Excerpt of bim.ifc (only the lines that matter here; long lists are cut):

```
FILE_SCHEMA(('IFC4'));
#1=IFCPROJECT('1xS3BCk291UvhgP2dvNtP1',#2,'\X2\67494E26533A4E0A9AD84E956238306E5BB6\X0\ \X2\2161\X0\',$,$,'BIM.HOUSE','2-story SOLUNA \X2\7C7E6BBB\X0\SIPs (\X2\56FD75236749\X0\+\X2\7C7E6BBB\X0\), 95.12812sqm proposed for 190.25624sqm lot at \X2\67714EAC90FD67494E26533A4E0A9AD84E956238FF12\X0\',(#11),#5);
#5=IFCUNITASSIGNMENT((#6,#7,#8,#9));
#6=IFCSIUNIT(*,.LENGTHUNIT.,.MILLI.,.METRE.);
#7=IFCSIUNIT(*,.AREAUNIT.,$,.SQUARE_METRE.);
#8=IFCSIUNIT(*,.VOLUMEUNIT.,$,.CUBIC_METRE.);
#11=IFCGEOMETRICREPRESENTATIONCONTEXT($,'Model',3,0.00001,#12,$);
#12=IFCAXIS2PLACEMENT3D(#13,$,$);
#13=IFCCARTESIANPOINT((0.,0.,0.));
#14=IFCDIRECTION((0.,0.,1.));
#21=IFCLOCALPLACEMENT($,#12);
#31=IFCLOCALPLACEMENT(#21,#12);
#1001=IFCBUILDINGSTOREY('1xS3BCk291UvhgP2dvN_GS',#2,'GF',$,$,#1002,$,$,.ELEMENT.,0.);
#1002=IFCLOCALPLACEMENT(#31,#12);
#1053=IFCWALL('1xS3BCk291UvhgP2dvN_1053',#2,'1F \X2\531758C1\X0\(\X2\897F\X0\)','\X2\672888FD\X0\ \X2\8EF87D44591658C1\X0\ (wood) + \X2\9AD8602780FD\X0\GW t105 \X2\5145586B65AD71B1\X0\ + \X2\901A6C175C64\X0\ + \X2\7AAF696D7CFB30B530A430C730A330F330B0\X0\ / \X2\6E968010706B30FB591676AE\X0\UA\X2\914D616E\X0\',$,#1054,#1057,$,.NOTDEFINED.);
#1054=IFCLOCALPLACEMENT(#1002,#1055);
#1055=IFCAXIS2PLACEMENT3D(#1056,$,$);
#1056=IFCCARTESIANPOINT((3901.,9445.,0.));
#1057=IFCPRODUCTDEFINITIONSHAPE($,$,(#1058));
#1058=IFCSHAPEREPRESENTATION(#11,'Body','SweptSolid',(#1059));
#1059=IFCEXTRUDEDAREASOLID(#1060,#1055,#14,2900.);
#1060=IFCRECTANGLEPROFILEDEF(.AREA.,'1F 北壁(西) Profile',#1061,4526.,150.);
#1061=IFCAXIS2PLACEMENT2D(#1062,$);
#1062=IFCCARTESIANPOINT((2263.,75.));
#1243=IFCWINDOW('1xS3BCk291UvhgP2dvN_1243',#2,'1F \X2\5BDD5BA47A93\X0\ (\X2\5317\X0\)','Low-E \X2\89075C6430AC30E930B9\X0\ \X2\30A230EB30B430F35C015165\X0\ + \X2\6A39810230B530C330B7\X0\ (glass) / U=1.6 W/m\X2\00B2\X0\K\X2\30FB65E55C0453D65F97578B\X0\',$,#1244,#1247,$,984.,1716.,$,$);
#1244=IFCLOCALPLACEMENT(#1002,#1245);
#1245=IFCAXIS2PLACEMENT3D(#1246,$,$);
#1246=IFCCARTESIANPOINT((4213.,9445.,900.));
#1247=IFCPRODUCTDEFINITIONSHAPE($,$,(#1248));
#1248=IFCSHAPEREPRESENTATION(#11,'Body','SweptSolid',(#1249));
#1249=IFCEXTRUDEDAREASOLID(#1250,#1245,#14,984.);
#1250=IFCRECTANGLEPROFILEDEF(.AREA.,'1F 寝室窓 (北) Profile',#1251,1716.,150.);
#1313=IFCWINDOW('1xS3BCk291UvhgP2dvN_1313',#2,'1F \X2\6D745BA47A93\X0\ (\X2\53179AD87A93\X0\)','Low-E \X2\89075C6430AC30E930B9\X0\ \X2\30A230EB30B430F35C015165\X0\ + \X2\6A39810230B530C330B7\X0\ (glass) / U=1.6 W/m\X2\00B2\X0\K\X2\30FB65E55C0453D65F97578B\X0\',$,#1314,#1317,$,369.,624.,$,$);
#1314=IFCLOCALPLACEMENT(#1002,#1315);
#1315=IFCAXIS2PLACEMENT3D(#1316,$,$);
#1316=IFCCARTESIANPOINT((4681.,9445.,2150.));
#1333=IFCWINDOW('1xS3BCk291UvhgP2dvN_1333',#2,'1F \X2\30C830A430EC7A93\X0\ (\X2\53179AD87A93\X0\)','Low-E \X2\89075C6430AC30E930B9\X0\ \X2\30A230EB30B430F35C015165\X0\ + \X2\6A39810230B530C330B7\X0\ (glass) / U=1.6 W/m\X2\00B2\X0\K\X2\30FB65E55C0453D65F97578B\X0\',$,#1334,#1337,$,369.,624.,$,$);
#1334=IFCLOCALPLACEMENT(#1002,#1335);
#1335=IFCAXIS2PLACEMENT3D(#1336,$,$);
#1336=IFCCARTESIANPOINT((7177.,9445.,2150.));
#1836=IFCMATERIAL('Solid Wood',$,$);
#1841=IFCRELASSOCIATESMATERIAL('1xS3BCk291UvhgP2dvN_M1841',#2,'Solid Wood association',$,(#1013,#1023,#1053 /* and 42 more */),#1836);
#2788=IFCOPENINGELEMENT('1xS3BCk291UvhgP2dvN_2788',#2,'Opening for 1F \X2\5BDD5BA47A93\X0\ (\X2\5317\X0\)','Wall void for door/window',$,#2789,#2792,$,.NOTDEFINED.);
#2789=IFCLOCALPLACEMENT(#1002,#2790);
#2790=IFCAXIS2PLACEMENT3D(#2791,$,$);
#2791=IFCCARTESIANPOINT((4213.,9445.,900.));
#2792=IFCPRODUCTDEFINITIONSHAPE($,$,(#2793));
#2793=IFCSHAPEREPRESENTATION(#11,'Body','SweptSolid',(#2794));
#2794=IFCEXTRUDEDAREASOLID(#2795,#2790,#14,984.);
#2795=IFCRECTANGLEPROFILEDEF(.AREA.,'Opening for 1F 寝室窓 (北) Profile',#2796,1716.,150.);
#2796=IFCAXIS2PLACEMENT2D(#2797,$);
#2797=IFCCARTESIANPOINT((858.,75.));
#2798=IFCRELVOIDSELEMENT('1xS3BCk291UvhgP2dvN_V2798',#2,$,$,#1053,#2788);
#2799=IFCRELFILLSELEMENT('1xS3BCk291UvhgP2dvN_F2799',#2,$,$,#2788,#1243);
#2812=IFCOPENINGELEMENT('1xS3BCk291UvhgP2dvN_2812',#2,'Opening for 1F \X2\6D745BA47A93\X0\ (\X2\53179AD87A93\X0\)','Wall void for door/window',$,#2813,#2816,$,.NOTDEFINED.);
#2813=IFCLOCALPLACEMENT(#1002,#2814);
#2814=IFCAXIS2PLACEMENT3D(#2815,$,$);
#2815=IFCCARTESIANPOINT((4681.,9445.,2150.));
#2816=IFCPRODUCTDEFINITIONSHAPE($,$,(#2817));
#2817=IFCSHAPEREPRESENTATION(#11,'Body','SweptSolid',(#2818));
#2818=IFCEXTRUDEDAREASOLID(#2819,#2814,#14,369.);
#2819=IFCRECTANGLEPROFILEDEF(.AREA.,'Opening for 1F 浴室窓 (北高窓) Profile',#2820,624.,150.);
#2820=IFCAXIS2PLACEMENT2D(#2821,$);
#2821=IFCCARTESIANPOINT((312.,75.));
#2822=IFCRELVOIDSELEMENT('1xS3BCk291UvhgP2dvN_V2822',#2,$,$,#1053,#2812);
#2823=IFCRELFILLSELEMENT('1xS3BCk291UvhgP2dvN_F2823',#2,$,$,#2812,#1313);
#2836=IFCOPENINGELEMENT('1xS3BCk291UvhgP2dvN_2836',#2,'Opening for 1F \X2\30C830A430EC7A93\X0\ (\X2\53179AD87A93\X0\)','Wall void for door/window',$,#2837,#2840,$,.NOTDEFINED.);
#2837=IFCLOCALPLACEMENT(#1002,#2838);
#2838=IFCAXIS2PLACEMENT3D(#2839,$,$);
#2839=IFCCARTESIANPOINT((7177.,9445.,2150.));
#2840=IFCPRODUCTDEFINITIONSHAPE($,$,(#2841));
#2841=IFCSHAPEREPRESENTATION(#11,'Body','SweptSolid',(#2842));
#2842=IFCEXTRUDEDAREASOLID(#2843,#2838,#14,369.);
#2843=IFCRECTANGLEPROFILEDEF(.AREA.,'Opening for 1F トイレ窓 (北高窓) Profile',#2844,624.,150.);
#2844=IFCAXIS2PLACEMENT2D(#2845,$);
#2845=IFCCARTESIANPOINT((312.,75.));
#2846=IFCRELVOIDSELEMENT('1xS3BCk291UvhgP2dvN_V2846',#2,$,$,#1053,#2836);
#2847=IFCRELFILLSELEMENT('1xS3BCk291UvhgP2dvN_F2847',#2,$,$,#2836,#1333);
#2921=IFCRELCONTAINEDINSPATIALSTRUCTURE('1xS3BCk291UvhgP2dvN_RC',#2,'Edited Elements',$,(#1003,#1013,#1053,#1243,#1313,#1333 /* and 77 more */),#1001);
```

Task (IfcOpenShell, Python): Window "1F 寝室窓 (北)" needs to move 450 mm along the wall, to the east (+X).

```python
import ifcopenshell
import ifcopenshell.api.geometry
import ifcopenshell.util.placement

model = ifcopenshell.open("bim.ifc")

window = model.by_guid("1xS3BCk291UvhgP2dvN_1243")
opening = window.FillsVoids[0].RelatingOpeningElement
wall = opening.VoidsElements[0].RelatingBuildingElement

wall_matrix = ifcopenshell.util.placement.get_local_placement(wall.ObjectPlacement)
shift = wall_matrix[:3, 0] * 450.0
before = ifcopenshell.util.placement.get_local_placement(window.ObjectPlacement)[:3, 3].copy()

# The window is not placed relative to its opening, so move both.
for product in (opening, window):
    matrix = ifcopenshell.util.placement.get_local_placement(product.ObjectPlacement)
    matrix[:3, 3] += shift
    ifcopenshell.api.geometry.edit_object_placement(model, product=product, matrix=matrix, is_si=False)

after = ifcopenshell.util.placement.get_local_placement(window.ObjectPlacement)[:3, 3]
print("window moved by", (after - before).round(3) + 0.0)

model.write("bim_edited.ifc")
```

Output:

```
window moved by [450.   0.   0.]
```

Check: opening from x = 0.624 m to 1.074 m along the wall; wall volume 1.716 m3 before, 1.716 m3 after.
